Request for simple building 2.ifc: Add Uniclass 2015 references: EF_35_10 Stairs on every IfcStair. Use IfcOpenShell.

First a look at what the model holds.

```python
import ifcopenshell

model = ifcopenshell.open("simple building 2.ifc")
print(model.schema)
print("classifications:", [c.Name for c in model.by_type("IfcClassification")])
for ifc_class in ("IfcDoor", "IfcRoof", "IfcStair", "IfcWall", "IfcWindow"):
    print(ifc_class, len(model.by_type(ifc_class)))
```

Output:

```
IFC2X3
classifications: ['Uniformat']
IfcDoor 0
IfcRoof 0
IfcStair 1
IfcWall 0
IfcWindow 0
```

```python
import ifcopenshell
import ifcopenshell.api.classification

model = ifcopenshell.open("simple building 2.ifc")

# IFC2X3 requires Source and Edition and has no link from the project to the system.
system = model.create_entity("IfcClassification", Source="NBS", Edition="2015", Name="Uniclass 2015")

codes = {
    "IfcStair": ("EF_35_10", "Stairs"),
}
for ifc_class, (code, name) in codes.items():
    products = model.by_type(ifc_class)
    ifcopenshell.api.classification.add_reference(
        model, products=products, classification=system, identification=code, name=name
    )
    print(code, len(products))

model.write("simple building 2-out.ifc")
```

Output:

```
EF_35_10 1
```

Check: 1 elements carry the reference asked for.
